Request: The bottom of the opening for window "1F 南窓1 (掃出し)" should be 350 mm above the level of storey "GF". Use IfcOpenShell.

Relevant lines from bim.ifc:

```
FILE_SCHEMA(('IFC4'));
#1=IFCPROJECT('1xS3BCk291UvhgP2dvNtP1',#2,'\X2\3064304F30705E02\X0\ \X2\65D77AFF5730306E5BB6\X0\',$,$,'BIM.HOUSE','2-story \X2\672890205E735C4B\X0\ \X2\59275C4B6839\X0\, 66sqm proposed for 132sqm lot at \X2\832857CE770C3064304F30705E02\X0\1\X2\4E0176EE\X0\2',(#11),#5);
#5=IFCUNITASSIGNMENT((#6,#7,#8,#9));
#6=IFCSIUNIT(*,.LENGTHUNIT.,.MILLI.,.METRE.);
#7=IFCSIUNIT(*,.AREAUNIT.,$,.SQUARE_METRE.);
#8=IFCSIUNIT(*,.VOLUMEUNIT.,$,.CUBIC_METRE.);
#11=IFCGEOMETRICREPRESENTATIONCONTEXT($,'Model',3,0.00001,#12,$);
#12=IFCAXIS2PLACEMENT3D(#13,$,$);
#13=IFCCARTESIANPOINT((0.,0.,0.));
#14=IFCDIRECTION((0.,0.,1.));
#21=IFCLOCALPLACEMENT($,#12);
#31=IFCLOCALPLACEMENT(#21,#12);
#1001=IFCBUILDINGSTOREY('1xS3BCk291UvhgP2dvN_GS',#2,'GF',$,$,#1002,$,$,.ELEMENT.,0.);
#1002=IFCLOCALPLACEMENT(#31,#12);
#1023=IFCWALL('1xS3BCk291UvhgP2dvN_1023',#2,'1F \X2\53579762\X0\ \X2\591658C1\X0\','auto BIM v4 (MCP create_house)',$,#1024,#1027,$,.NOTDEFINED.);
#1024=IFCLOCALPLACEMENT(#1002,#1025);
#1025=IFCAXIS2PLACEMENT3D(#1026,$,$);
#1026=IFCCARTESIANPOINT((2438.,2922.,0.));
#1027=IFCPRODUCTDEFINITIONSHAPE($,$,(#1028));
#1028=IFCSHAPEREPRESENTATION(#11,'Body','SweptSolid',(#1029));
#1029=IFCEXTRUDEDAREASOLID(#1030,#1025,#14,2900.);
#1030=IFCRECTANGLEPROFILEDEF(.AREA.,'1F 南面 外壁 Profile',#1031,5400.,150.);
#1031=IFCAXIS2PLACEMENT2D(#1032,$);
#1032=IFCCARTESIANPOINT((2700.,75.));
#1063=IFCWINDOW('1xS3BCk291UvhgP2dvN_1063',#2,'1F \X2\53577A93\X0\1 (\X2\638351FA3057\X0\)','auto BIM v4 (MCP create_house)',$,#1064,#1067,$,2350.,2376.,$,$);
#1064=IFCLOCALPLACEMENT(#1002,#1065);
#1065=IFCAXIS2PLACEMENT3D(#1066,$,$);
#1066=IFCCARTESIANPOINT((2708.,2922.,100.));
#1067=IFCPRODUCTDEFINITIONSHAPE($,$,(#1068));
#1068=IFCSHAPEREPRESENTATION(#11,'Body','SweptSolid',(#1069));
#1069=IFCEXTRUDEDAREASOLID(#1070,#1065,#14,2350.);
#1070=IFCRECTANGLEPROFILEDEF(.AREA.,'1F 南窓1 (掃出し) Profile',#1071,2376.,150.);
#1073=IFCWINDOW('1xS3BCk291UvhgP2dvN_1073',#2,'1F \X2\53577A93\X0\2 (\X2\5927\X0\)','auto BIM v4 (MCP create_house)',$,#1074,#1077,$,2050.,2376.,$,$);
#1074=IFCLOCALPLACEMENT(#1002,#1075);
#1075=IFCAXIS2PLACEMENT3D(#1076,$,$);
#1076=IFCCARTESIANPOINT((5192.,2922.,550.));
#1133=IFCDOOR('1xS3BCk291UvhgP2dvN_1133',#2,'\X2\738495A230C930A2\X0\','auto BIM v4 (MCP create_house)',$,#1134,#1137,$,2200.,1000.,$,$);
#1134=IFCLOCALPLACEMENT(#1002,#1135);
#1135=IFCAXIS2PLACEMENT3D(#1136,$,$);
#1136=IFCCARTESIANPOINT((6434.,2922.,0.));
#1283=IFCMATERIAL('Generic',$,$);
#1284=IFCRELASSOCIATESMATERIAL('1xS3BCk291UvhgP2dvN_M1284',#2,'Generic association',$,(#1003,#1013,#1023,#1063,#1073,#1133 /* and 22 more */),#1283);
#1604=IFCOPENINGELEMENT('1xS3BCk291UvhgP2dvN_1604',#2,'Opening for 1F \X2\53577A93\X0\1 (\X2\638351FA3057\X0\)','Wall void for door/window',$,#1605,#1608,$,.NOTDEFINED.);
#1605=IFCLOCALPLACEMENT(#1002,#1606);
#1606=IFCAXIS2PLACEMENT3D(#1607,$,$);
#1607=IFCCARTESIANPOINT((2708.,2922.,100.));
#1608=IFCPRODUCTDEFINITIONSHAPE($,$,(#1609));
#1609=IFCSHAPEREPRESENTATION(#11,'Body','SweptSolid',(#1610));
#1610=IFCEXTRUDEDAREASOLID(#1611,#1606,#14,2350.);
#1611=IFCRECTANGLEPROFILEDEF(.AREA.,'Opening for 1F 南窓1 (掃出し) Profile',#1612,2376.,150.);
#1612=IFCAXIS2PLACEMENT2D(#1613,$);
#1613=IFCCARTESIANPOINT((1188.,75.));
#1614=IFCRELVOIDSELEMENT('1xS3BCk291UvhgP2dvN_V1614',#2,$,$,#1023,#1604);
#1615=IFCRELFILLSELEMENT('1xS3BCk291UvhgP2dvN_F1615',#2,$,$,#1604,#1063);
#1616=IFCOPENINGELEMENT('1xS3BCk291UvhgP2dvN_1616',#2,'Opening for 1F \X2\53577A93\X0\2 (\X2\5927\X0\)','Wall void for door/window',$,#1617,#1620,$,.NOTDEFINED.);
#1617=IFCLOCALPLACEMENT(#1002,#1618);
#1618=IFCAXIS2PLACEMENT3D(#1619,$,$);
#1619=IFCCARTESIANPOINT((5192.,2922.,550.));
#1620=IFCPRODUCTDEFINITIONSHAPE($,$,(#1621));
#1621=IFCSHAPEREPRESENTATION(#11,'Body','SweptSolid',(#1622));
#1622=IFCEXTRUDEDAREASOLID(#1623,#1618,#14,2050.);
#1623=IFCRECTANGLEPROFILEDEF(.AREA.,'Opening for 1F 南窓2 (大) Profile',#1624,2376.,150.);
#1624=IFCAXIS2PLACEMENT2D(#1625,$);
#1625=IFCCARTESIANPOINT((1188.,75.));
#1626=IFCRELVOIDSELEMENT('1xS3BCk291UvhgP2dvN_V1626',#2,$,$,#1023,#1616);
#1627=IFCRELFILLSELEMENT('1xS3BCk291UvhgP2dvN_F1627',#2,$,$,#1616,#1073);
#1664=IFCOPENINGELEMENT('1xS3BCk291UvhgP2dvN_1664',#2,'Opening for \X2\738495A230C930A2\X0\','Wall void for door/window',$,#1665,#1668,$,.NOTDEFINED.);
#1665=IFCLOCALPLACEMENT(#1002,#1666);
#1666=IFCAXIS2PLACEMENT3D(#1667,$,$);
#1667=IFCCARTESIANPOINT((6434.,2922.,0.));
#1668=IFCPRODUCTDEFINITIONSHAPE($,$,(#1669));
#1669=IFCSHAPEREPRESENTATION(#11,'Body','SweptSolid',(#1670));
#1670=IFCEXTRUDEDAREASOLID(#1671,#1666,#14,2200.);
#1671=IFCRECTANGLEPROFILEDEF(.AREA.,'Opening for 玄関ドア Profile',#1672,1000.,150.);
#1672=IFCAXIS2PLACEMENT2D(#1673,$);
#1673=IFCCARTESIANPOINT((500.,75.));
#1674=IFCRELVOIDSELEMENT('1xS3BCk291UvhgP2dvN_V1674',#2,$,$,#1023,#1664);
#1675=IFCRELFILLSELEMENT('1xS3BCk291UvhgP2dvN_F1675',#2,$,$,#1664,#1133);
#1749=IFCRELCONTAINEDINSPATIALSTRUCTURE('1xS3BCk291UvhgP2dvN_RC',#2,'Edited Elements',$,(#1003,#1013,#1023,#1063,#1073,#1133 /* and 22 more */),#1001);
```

```python
import numpy as np
import ifcopenshell
import ifcopenshell.api.geometry
import ifcopenshell.geom
import ifcopenshell.util.element
import ifcopenshell.util.placement
import ifcopenshell.util.shape
import ifcopenshell.util.unit

model = ifcopenshell.open("bim.ifc")
unit_scale = ifcopenshell.util.unit.calculate_unit_scale(model)

window = model.by_guid("1xS3BCk291UvhgP2dvN_1063")
opening = window.FillsVoids[0].RelatingOpeningElement
storey = ifcopenshell.util.element.get_container(window, ifc_class="IfcBuildingStorey")
level = ifcopenshell.util.placement.get_local_placement(storey.ObjectPlacement)[2, 3]

# The opening's origin need not be at the sill, so measure its lowest point.
shape = ifcopenshell.geom.create_shape(ifcopenshell.geom.settings(), opening)
bottom = ifcopenshell.util.shape.get_shape_bottom_elevation(shape, shape.geometry) / unit_scale
dz = level + 350.0 - bottom

shift = np.array([0.0, 0.0, dz])
# The window is not placed relative to its opening, so move both.
for product in (opening, window):
    matrix = ifcopenshell.util.placement.get_local_placement(product.ObjectPlacement)
    matrix[:3, 3] += shift
    ifcopenshell.api.geometry.edit_object_placement(model, product=product, matrix=matrix, is_si=False)

print(f"moved by {dz * unit_scale:+.3f} m")

model.write("bim_v2.ifc")
```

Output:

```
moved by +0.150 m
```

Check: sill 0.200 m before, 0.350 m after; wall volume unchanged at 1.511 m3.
